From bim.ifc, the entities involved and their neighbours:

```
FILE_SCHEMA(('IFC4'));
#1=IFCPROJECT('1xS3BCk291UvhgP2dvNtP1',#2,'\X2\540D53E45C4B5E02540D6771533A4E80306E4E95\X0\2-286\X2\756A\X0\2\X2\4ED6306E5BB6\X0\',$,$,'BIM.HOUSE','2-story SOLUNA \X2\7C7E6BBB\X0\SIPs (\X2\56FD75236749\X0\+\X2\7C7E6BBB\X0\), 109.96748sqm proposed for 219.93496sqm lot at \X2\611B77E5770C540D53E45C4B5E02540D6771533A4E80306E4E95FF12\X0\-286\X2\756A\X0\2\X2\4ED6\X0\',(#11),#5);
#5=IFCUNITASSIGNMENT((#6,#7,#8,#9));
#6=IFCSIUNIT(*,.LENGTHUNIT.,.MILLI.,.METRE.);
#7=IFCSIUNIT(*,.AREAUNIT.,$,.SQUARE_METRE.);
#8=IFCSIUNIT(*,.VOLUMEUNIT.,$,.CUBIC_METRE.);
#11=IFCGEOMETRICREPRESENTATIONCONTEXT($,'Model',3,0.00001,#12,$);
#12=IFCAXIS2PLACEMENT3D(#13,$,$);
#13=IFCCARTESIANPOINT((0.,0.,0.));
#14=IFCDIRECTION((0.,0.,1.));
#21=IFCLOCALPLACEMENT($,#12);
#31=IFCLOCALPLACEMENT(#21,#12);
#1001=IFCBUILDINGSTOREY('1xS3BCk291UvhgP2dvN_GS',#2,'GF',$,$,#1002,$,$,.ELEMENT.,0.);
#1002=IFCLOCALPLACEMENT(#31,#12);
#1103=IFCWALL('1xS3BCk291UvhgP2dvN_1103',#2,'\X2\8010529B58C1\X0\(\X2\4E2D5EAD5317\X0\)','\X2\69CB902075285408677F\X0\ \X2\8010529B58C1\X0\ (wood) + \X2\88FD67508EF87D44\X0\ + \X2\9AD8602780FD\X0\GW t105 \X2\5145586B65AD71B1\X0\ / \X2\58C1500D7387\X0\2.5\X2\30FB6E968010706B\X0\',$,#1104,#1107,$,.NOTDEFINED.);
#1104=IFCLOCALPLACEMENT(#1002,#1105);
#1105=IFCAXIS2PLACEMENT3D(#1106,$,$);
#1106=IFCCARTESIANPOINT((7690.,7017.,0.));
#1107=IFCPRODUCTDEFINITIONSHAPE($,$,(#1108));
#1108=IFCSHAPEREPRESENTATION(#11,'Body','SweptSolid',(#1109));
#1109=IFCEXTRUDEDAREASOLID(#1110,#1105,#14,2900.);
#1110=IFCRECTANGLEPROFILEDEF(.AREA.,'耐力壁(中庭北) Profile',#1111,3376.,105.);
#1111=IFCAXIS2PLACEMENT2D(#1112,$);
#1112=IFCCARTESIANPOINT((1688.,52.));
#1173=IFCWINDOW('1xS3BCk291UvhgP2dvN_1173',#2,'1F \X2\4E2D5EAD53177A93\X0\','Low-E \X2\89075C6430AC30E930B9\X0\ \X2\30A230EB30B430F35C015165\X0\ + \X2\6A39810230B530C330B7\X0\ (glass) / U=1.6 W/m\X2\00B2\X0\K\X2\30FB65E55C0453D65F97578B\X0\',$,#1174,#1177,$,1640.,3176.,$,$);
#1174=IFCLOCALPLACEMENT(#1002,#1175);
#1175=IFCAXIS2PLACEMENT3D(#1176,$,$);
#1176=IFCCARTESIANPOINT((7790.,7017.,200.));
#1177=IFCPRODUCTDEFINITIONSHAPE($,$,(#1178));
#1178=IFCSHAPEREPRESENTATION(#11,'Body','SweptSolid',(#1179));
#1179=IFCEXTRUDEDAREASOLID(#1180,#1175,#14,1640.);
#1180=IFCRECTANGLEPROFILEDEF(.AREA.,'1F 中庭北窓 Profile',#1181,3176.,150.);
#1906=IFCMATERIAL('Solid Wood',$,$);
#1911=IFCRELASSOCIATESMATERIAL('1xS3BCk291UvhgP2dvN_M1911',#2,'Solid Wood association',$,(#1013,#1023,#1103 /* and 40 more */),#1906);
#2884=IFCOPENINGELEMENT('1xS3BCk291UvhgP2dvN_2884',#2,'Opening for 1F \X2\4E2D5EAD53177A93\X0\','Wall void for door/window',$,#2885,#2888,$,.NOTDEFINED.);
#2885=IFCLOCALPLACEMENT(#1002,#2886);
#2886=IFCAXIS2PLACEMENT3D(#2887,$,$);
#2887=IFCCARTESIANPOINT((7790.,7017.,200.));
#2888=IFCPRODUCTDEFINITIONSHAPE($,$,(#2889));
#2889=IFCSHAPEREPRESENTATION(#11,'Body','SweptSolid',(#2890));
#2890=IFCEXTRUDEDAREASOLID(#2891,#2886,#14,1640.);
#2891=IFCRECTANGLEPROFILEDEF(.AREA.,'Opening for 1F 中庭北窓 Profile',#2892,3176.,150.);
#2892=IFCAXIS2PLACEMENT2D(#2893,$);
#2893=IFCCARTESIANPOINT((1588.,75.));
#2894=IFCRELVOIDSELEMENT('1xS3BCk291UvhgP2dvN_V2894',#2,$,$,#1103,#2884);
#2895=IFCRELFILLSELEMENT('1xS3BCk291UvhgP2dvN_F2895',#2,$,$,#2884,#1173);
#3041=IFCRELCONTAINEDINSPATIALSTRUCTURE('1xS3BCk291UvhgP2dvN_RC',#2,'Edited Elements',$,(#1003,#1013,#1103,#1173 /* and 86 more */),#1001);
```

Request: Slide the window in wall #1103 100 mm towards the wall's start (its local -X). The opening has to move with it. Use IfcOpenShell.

```python
import ifcopenshell
import ifcopenshell.api.geometry
import ifcopenshell.util.placement

model = ifcopenshell.open("bim.ifc")

window = model.by_guid("1xS3BCk291UvhgP2dvN_1173")
opening = window.FillsVoids[0].RelatingOpeningElement
wall = opening.VoidsElements[0].RelatingBuildingElement

wall_matrix = ifcopenshell.util.placement.get_local_placement(wall.ObjectPlacement)
shift = wall_matrix[:3, 0] * -100.0
before = ifcopenshell.util.placement.get_local_placement(window.ObjectPlacement)[:3, 3].copy()

# The window is not placed relative to its opening, so move both.
for product in (opening, window):
    matrix = ifcopenshell.util.placement.get_local_placement(product.ObjectPlacement)
    matrix[:3, 3] += shift
    ifcopenshell.api.geometry.edit_object_placement(model, product=product, matrix=matrix, is_si=False)

after = ifcopenshell.util.placement.get_local_placement(window.ObjectPlacement)[:3, 3]
print("window moved by", (after - before).round(3) + 0.0)

model.write("bim_v2.ifc")
```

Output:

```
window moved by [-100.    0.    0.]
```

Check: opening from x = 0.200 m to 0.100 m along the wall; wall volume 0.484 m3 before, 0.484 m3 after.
